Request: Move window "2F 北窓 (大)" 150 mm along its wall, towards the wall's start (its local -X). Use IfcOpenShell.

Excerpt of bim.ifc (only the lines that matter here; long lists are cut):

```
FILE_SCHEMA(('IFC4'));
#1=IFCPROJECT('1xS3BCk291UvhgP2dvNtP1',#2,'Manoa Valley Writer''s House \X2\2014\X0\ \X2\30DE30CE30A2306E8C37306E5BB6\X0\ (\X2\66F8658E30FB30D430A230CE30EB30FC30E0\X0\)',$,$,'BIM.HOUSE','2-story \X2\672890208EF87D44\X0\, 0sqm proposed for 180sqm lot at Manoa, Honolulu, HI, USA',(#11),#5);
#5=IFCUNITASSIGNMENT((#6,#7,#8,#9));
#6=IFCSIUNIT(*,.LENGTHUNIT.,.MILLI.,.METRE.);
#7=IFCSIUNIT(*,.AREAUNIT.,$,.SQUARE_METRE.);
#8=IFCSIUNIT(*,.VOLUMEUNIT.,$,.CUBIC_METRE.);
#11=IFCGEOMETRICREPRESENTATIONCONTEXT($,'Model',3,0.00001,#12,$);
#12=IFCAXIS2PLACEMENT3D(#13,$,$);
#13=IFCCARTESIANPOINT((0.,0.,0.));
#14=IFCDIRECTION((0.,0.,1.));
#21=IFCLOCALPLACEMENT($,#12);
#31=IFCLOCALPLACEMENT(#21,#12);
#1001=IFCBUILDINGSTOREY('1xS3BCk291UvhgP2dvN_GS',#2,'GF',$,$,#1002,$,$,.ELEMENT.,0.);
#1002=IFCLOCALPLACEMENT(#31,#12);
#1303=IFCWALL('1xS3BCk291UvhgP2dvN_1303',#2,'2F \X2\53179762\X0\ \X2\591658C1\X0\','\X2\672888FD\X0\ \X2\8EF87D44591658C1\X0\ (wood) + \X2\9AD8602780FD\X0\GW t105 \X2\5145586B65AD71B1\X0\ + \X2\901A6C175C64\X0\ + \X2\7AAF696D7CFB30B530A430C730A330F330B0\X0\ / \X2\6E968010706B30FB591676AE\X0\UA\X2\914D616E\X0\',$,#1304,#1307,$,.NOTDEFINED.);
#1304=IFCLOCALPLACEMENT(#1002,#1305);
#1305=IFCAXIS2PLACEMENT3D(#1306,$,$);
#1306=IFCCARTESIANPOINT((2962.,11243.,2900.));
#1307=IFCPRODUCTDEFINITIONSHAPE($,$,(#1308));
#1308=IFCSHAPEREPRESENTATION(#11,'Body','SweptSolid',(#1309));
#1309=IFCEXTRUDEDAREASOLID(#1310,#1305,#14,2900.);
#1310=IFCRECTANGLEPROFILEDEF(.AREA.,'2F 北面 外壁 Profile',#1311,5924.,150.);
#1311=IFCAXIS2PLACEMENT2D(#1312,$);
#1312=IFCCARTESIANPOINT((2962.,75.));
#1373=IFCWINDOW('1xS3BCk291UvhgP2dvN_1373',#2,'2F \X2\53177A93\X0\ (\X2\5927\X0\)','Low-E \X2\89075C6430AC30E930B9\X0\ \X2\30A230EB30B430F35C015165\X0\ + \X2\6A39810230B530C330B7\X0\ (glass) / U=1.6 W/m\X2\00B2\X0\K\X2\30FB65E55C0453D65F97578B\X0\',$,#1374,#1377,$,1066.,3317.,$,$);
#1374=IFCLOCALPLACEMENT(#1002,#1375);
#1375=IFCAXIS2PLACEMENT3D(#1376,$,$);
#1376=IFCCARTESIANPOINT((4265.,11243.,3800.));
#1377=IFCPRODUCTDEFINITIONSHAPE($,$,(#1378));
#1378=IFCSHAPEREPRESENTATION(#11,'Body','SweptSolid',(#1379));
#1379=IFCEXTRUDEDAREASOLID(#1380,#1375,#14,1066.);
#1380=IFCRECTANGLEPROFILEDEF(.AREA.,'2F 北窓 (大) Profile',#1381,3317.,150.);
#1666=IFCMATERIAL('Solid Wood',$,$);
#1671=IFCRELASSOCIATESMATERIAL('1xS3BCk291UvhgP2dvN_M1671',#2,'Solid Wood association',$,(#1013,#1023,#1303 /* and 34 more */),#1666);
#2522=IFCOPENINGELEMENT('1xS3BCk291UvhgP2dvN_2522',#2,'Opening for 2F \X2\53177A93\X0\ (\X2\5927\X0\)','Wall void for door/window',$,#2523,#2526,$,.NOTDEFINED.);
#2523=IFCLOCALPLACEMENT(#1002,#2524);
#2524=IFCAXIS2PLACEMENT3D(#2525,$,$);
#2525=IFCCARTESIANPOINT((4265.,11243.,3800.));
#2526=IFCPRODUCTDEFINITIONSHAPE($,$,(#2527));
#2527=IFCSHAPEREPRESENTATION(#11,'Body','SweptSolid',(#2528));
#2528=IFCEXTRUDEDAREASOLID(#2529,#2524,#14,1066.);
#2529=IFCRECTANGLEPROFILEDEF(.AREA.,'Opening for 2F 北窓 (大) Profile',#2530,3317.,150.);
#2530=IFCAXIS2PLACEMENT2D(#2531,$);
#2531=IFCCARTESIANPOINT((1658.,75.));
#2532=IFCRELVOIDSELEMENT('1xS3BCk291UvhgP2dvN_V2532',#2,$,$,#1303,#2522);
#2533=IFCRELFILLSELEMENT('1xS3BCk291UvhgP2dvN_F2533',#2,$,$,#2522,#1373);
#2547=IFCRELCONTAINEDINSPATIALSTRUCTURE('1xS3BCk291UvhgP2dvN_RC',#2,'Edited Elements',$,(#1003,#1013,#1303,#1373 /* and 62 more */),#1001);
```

```python
import ifcopenshell
import ifcopenshell.api.geometry
import ifcopenshell.util.placement
import ifcopenshell.util.unit

model = ifcopenshell.open("bim.ifc")
unit_scale = ifcopenshell.util.unit.calculate_unit_scale(model)

window = model.by_guid("1xS3BCk291UvhgP2dvN_1373")
opening = window.FillsVoids[0].RelatingOpeningElement
wall = opening.VoidsElements[0].RelatingBuildingElement

wall_matrix = ifcopenshell.util.placement.get_local_placement(wall.ObjectPlacement)
shift = wall_matrix[:3, 0] * -0.15 / unit_scale
before = ifcopenshell.util.placement.get_local_placement(window.ObjectPlacement)[:3, 3].copy()

# The window is not placed relative to its opening, so move both.
for product in (opening, window):
    matrix = ifcopenshell.util.placement.get_local_placement(product.ObjectPlacement)
    matrix[:3, 3] += shift
    ifcopenshell.api.geometry.edit_object_placement(model, product=product, matrix=matrix, is_si=False)

after = ifcopenshell.util.placement.get_local_placement(window.ObjectPlacement)[:3, 3]
print("window moved by", (after - before).round(3) + 0.0)

model.write("bim_edited.ifc")
```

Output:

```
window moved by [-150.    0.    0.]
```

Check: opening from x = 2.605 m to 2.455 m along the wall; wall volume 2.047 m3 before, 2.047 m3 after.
